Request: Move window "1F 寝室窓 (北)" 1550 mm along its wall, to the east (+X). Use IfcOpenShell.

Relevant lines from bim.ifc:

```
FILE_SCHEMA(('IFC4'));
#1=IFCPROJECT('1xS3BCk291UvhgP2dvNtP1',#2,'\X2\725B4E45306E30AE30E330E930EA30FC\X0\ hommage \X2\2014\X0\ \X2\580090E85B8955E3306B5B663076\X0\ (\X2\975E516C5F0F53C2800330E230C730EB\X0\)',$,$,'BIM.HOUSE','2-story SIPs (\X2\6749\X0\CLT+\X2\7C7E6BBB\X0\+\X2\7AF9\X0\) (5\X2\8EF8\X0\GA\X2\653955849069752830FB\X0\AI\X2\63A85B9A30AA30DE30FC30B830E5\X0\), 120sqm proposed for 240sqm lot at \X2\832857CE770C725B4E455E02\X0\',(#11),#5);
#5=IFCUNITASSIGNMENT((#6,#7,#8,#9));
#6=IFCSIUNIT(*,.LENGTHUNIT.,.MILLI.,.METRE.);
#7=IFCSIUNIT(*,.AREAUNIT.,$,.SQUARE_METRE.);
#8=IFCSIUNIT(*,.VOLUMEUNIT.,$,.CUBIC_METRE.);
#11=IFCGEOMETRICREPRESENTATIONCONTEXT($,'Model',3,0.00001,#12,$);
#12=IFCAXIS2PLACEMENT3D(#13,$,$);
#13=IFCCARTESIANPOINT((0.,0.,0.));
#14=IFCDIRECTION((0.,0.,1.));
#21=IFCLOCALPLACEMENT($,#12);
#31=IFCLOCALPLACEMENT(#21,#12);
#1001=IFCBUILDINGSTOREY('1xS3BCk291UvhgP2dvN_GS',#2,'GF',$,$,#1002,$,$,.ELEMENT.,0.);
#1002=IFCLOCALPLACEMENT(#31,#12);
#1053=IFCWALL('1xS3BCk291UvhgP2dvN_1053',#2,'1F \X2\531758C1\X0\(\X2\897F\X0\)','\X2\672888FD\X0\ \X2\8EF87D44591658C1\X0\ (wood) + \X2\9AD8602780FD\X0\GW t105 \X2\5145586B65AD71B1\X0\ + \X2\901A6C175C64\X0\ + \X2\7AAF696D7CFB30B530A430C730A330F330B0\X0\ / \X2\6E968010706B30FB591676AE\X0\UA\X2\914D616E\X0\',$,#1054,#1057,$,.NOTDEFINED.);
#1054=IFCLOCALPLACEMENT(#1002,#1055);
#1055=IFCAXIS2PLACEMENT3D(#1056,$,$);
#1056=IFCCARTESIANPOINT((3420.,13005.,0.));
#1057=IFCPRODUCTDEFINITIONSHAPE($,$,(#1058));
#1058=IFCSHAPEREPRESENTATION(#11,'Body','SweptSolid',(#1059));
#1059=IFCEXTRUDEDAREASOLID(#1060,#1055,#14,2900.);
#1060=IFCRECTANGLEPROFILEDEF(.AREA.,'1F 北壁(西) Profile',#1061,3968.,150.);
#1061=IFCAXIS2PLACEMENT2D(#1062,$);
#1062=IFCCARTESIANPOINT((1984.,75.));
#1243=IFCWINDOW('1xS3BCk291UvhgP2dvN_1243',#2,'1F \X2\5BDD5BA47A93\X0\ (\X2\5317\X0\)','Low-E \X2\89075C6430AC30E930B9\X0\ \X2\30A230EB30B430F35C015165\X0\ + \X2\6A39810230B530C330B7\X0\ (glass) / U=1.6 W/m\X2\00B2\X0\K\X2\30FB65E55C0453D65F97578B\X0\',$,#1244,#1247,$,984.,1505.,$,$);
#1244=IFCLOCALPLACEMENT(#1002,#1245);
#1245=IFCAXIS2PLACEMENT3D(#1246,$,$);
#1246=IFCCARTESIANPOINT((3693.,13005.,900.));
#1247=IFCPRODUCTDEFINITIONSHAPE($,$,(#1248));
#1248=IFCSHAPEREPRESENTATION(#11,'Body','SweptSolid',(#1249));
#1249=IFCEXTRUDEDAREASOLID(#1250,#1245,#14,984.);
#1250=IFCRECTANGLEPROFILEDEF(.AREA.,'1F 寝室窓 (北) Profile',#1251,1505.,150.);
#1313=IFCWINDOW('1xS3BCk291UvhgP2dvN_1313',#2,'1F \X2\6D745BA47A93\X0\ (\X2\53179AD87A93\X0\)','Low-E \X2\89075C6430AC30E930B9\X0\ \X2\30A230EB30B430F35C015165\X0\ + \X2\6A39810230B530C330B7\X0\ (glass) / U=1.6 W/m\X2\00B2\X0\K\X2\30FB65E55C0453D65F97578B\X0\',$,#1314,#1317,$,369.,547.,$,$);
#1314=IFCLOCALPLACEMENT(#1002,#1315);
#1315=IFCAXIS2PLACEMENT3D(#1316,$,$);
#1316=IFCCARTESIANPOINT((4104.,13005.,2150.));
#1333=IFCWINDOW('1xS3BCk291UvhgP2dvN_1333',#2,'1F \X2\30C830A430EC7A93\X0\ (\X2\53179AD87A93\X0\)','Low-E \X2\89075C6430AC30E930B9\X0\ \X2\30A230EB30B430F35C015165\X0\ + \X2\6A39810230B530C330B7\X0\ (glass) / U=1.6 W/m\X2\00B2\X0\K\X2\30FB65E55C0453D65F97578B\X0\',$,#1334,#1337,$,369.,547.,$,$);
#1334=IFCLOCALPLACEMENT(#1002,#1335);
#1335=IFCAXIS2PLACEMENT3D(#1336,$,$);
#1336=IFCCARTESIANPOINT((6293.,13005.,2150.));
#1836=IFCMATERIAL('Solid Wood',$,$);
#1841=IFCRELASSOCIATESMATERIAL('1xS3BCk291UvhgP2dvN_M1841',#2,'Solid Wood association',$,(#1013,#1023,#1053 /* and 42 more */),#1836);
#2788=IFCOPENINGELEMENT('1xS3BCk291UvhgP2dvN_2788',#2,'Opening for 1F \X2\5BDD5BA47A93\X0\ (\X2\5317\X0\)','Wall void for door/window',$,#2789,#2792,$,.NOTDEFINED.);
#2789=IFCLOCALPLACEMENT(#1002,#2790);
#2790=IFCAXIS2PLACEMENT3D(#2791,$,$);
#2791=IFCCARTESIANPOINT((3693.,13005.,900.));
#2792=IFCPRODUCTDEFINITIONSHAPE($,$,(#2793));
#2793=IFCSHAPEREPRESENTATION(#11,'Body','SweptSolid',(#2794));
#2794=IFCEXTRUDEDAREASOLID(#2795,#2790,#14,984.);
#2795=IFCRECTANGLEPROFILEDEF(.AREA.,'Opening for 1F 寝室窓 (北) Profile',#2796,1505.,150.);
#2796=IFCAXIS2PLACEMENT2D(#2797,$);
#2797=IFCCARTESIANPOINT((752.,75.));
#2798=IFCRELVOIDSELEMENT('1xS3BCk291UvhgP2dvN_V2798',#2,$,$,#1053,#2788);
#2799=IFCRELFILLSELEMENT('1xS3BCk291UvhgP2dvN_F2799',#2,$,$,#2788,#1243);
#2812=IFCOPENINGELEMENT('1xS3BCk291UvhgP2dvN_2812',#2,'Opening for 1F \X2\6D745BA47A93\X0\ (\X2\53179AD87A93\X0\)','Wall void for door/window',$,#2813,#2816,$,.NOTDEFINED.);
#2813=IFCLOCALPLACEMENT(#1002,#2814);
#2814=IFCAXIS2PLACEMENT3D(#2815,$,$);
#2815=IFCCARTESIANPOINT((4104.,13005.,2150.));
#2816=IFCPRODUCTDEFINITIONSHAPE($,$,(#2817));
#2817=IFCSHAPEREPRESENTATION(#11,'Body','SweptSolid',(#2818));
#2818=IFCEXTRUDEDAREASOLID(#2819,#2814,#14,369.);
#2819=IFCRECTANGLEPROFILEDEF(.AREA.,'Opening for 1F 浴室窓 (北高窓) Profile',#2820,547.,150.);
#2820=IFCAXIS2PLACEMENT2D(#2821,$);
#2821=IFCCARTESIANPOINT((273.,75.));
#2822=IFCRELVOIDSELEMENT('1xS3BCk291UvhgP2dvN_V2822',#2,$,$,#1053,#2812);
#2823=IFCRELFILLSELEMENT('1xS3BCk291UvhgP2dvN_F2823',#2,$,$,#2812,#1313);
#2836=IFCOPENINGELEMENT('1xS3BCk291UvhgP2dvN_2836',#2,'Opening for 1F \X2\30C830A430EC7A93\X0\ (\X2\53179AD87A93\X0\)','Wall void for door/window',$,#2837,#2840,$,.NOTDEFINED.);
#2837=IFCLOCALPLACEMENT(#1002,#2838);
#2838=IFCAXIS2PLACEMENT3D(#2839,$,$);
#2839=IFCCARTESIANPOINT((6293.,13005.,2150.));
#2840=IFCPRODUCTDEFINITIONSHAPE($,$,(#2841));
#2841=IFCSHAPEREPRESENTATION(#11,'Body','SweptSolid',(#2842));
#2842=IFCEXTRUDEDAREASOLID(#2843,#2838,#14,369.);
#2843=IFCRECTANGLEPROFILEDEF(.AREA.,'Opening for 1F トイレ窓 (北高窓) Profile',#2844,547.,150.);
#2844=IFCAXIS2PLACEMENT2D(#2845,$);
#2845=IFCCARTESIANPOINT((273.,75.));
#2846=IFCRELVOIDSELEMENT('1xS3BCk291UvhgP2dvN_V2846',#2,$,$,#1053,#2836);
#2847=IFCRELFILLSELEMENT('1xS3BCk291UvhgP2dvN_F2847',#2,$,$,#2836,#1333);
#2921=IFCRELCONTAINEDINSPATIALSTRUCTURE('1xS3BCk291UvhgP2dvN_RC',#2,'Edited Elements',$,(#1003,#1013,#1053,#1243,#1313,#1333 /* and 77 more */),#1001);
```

```python
import ifcopenshell
import ifcopenshell.api.geometry
import ifcopenshell.util.placement

model = ifcopenshell.open("bim.ifc")

window = model.by_guid("1xS3BCk291UvhgP2dvN_1243")
opening = window.FillsVoids[0].RelatingOpeningElement
wall = opening.VoidsElements[0].RelatingBuildingElement

wall_matrix = ifcopenshell.util.placement.get_local_placement(wall.ObjectPlacement)
shift = wall_matrix[:3, 0] * 1550.0
before = ifcopenshell.util.placement.get_local_placement(window.ObjectPlacement)[:3, 3].copy()

# The window is not placed relative to its opening, so move both.
for product in (opening, window):
    matrix = ifcopenshell.util.placement.get_local_placement(product.ObjectPlacement)
    matrix[:3, 3] += shift
    ifcopenshell.api.geometry.edit_object_placement(model, product=product, matrix=matrix, is_si=False)

after = ifcopenshell.util.placement.get_local_placement(window.ObjectPlacement)[:3, 3]
print("window moved by", (after - before).round(3) + 0.0)

model.write("bim_edited.ifc")
```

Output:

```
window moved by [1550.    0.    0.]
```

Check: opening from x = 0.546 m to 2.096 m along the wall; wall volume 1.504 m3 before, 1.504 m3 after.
